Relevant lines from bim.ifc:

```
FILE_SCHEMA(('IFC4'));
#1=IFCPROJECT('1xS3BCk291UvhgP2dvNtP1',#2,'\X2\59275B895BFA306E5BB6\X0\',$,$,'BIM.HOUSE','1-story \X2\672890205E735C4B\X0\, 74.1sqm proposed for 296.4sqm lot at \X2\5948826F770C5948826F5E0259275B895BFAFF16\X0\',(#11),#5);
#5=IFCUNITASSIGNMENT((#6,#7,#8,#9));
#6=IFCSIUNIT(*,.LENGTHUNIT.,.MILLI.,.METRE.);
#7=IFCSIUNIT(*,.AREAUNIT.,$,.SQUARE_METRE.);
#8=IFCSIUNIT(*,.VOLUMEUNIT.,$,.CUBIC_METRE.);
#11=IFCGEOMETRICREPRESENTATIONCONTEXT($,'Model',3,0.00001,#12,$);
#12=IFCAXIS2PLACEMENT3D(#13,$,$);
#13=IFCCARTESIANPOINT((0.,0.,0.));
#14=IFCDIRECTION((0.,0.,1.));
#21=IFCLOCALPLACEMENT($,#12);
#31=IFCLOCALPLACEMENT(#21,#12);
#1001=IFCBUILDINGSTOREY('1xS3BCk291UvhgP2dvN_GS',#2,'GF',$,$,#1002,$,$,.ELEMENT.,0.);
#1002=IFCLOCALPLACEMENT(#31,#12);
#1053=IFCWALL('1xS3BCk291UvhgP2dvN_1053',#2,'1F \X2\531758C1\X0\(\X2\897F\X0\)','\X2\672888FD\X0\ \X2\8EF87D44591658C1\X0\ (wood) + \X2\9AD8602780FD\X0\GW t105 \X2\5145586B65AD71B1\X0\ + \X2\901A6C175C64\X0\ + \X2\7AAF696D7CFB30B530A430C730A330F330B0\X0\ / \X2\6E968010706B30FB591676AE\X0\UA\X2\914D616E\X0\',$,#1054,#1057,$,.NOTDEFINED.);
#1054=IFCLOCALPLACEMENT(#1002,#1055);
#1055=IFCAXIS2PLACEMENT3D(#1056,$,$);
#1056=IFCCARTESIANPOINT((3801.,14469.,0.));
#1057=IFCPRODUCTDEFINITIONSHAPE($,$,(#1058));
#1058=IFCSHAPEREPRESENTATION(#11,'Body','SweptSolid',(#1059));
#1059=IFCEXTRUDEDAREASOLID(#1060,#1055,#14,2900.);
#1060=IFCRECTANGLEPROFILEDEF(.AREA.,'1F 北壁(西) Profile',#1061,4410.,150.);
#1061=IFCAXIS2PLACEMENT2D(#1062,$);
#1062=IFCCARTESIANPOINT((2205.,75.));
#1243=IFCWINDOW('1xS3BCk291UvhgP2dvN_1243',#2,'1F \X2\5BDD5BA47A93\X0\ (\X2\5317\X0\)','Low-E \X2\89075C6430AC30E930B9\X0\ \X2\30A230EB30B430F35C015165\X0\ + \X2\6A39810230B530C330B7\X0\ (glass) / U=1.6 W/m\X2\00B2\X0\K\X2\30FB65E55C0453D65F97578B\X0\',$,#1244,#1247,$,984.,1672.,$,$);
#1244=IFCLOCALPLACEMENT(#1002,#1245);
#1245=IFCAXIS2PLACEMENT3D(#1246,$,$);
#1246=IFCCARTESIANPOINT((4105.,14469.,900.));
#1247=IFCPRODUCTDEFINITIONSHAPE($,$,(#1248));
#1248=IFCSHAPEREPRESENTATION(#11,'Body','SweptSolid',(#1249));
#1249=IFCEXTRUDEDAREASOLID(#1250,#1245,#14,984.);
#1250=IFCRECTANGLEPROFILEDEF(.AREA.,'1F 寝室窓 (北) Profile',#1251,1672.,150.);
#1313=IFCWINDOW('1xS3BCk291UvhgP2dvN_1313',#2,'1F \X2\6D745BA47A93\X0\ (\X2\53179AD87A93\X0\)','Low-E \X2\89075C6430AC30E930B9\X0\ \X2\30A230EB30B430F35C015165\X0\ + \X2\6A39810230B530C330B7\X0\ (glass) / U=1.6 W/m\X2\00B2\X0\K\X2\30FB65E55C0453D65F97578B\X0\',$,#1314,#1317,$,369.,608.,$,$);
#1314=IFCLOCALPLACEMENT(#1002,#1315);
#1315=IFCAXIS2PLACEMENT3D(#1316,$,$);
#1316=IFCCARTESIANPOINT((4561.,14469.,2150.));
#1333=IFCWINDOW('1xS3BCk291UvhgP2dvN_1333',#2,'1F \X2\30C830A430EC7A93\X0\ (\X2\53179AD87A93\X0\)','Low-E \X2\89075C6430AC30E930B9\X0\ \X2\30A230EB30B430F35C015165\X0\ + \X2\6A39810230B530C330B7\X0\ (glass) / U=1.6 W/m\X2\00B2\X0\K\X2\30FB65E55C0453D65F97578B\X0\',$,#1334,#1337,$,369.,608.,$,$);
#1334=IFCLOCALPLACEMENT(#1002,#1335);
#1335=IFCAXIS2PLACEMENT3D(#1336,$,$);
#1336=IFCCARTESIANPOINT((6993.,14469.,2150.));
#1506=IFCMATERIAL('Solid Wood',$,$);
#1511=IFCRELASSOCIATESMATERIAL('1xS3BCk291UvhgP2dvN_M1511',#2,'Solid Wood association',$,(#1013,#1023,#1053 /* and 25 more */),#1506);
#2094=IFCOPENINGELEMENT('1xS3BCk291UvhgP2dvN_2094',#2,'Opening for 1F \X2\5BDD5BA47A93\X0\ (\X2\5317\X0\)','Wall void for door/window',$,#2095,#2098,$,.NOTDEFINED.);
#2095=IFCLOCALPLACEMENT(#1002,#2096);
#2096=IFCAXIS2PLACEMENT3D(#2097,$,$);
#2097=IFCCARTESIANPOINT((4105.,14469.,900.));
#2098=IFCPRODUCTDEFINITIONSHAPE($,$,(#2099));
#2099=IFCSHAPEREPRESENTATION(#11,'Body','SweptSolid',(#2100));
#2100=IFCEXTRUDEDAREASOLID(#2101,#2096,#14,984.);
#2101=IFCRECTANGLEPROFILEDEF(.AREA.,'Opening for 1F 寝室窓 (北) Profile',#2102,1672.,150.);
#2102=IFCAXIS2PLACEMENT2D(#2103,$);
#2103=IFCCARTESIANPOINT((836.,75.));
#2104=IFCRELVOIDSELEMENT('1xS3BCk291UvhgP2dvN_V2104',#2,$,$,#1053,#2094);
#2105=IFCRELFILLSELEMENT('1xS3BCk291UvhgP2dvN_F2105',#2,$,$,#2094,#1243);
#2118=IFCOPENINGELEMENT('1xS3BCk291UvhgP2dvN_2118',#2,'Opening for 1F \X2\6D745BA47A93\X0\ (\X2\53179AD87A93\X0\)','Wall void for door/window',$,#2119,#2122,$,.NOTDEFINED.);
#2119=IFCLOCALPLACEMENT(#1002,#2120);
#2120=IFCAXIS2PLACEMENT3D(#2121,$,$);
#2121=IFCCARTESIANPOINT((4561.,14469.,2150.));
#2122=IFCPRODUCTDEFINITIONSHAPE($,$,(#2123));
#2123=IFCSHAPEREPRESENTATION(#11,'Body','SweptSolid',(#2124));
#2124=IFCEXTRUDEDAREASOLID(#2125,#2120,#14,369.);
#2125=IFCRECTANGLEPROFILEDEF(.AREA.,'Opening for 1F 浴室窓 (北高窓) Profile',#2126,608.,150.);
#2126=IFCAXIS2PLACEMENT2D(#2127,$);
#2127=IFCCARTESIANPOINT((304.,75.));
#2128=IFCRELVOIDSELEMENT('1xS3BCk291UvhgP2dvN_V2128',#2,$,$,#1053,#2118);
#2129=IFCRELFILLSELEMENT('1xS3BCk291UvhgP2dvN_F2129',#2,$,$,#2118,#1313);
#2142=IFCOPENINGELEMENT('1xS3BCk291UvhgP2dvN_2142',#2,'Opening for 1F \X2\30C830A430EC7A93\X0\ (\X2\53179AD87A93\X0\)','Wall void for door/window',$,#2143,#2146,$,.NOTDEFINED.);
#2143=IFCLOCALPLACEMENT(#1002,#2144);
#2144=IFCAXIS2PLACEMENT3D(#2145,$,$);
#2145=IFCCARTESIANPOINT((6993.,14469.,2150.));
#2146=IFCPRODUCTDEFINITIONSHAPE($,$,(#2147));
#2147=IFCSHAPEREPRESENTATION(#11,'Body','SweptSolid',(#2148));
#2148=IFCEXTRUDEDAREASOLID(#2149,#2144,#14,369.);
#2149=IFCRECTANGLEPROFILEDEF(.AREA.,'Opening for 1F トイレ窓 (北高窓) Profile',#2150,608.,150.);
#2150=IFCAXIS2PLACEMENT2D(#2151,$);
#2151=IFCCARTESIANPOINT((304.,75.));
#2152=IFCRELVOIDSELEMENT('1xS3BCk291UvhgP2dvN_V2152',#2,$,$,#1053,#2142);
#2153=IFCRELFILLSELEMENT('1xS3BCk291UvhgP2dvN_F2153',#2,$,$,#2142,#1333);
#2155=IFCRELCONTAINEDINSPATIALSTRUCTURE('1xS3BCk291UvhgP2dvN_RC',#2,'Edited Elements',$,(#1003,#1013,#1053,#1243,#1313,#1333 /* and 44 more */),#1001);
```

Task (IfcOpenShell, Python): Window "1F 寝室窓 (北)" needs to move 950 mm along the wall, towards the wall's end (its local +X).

```python
import ifcopenshell
import ifcopenshell.api.geometry
import ifcopenshell.util.placement
import ifcopenshell.util.unit

model = ifcopenshell.open("bim.ifc")
unit_scale = ifcopenshell.util.unit.calculate_unit_scale(model)

window = model.by_guid("1xS3BCk291UvhgP2dvN_1243")
opening = window.FillsVoids[0].RelatingOpeningElement
wall = opening.VoidsElements[0].RelatingBuildingElement

wall_matrix = ifcopenshell.util.placement.get_local_placement(wall.ObjectPlacement)
shift = wall_matrix[:3, 0] * 0.95 / unit_scale
before = ifcopenshell.util.placement.get_local_placement(window.ObjectPlacement)[:3, 3].copy()

# The window is not placed relative to its opening, so move both.
for product in (opening, window):
    matrix = ifcopenshell.util.placement.get_local_placement(product.ObjectPlacement)
    matrix[:3, 3] += shift
    ifcopenshell.api.geometry.edit_object_placement(model, product=product, matrix=matrix, is_si=False)

after = ifcopenshell.util.placement.get_local_placement(window.ObjectPlacement)[:3, 3]
print("window moved by", (after - before).round(3) + 0.0)

model.write("bim_rev.ifc")
```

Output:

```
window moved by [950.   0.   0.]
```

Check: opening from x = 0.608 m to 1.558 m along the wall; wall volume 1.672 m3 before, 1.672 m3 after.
